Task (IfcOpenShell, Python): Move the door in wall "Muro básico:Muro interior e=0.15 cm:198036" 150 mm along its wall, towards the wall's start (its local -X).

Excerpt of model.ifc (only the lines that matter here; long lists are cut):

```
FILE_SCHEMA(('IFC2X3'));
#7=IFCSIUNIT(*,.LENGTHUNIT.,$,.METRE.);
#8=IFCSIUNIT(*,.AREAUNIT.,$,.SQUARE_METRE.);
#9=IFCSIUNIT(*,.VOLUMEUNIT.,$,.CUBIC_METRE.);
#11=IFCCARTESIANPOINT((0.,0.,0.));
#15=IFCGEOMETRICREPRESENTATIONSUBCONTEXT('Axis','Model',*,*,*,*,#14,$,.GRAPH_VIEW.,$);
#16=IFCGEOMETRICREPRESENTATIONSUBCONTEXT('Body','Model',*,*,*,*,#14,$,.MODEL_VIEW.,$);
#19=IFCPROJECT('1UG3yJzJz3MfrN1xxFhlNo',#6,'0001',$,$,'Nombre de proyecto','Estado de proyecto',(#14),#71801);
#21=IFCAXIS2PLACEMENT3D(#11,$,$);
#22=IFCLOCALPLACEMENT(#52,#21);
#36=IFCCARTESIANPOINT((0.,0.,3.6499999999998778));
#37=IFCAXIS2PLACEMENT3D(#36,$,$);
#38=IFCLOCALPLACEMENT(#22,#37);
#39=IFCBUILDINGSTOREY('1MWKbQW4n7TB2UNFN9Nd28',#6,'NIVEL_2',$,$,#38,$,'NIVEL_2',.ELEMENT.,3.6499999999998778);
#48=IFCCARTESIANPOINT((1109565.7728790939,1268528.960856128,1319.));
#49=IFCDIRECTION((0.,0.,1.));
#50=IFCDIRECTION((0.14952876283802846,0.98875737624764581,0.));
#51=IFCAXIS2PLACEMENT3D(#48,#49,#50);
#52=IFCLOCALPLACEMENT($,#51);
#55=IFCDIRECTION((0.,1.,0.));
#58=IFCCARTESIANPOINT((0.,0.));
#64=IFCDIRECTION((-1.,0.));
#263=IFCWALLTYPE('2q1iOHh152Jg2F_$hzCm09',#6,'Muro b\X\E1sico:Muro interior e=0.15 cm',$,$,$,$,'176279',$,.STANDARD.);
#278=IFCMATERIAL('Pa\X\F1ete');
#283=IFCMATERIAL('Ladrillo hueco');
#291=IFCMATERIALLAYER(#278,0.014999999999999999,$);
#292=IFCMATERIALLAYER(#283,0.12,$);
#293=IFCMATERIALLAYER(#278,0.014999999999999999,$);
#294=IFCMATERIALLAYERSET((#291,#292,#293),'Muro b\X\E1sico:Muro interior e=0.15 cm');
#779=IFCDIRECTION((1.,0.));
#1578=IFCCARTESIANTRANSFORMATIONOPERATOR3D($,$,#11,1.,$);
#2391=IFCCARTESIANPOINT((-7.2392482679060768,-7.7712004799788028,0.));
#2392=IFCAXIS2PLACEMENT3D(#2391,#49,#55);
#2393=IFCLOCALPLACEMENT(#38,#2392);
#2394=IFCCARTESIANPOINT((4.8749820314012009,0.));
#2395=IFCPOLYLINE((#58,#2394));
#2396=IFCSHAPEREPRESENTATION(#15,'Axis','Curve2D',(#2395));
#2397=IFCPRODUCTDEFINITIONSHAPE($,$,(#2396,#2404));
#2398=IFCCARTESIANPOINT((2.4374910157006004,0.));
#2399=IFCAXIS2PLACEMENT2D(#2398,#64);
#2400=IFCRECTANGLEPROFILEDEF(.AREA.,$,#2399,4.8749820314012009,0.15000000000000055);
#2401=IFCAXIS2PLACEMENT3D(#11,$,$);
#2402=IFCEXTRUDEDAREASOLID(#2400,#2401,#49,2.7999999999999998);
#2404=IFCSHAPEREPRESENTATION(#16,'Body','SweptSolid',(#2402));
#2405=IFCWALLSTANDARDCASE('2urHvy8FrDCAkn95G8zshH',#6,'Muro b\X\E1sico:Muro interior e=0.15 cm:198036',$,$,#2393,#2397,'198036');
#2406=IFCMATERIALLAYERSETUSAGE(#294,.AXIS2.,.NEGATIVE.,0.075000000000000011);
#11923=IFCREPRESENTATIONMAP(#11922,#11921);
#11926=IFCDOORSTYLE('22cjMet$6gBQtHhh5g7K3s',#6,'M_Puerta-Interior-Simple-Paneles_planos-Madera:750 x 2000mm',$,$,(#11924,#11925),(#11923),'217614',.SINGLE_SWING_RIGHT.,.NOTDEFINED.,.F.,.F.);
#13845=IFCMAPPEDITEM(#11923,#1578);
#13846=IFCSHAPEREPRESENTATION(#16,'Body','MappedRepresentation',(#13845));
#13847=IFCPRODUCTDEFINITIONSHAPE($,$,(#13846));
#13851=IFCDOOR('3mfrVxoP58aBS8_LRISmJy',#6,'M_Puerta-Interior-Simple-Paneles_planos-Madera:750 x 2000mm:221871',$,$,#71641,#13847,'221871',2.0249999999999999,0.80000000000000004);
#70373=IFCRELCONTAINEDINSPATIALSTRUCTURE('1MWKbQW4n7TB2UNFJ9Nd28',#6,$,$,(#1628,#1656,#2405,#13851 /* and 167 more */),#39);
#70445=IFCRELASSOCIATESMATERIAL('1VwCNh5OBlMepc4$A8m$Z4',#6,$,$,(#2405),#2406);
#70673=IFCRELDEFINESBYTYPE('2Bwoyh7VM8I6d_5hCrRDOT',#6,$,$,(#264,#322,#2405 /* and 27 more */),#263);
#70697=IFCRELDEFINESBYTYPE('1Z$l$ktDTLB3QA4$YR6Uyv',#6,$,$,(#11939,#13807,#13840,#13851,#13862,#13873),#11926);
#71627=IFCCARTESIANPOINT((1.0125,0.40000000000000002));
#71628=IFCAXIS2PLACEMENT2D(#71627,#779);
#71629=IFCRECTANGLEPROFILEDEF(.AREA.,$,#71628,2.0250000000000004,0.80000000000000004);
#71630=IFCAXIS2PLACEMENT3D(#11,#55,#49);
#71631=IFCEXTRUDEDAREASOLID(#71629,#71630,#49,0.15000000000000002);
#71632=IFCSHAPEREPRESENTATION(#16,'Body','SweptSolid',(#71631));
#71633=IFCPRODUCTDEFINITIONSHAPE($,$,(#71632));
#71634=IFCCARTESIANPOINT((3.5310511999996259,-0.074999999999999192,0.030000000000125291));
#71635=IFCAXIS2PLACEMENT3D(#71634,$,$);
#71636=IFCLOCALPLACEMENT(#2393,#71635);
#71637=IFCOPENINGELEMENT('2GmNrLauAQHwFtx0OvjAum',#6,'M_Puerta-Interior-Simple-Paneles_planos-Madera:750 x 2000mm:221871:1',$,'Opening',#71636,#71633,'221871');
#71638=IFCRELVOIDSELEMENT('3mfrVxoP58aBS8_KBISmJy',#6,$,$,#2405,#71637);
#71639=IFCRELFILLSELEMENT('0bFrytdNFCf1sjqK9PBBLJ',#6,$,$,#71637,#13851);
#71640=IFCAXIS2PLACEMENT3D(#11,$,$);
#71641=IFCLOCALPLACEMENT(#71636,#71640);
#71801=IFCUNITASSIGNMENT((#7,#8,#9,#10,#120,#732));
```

```python
import ifcopenshell
import ifcopenshell.api.geometry
import ifcopenshell.util.placement

model = ifcopenshell.open("model.ifc")

door = model.by_guid("3mfrVxoP58aBS8_LRISmJy")
opening = door.FillsVoids[0].RelatingOpeningElement
wall = opening.VoidsElements[0].RelatingBuildingElement

wall_matrix = ifcopenshell.util.placement.get_local_placement(wall.ObjectPlacement)
shift = wall_matrix[:3, 0] * -0.15
before = ifcopenshell.util.placement.get_local_placement(door.ObjectPlacement)[:3, 3].copy()

# The door is placed relative to its opening, so it follows when the opening moves.
matrix = ifcopenshell.util.placement.get_local_placement(opening.ObjectPlacement)
matrix[:3, 3] += shift
ifcopenshell.api.geometry.edit_object_placement(
    model, product=opening, matrix=matrix, is_si=False, should_transform_children=True
)

after = ifcopenshell.util.placement.get_local_placement(door.ObjectPlacement)[:3, 3]
print("door moved by", (after - before).round(3) + 0.0)

model.write("model-out.ifc")
```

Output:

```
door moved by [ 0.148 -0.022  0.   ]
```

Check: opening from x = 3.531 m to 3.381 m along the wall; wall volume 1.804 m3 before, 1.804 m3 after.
